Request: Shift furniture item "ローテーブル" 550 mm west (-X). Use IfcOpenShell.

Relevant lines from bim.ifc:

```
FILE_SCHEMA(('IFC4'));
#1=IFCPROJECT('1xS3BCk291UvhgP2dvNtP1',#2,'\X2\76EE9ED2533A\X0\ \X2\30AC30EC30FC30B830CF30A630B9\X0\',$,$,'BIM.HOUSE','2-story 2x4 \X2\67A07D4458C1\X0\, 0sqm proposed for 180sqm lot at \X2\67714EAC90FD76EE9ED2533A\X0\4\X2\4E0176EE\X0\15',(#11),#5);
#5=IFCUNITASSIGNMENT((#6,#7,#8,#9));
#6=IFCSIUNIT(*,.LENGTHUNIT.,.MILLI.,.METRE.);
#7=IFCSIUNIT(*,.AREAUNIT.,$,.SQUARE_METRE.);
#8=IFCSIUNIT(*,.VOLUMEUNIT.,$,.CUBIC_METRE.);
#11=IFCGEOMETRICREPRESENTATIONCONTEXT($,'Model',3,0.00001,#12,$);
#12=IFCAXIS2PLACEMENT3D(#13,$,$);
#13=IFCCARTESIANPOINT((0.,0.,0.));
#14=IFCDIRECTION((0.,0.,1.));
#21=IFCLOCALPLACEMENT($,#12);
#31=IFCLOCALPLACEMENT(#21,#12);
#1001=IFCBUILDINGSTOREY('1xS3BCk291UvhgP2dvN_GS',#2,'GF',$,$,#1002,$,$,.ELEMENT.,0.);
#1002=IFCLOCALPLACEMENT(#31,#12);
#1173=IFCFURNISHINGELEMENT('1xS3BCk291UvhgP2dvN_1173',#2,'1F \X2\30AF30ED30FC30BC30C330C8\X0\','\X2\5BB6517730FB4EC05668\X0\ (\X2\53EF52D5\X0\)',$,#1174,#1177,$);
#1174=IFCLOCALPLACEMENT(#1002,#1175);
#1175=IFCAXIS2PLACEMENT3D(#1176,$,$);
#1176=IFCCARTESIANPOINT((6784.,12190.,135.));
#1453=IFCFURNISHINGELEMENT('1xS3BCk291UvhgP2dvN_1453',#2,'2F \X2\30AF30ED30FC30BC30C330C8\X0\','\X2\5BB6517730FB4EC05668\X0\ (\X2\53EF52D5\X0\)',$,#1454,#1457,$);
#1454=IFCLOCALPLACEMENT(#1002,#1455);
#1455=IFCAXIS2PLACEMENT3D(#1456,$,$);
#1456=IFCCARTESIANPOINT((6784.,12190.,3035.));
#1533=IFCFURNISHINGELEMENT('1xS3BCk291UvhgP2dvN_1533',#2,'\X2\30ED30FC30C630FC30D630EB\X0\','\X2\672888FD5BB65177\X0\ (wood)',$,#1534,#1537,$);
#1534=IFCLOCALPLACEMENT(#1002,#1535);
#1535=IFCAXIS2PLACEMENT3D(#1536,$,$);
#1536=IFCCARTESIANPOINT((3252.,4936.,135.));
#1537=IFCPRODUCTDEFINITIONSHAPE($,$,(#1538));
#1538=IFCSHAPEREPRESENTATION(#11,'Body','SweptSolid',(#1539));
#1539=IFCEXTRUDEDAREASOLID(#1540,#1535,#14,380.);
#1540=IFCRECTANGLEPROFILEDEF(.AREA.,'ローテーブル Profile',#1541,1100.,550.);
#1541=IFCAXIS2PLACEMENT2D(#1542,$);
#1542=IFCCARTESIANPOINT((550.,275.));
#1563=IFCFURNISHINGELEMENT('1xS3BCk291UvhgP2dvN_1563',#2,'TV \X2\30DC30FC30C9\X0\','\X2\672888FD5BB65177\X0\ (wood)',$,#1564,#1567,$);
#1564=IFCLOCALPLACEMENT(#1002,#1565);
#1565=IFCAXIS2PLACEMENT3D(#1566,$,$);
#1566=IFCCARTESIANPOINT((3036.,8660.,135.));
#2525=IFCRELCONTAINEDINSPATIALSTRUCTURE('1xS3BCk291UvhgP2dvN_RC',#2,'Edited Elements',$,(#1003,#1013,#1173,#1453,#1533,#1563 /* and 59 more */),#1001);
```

```python
import ifcopenshell
import ifcopenshell.api.geometry
import ifcopenshell.util.placement

model = ifcopenshell.open("bim.ifc")

item = model.by_guid("1xS3BCk291UvhgP2dvN_1533")
matrix = ifcopenshell.util.placement.get_local_placement(item.ObjectPlacement)
matrix[0, 3] -= 550.0
ifcopenshell.api.geometry.edit_object_placement(model, product=item, matrix=matrix, is_si=False)

print(ifcopenshell.util.placement.get_local_placement(item.ObjectPlacement).round(3) + 0.0)

model.write("bim-out.ifc")
```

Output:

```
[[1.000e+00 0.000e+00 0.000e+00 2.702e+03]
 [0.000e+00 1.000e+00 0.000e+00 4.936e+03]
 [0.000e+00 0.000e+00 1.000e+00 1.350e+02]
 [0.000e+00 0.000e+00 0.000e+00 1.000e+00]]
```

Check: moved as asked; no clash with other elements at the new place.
